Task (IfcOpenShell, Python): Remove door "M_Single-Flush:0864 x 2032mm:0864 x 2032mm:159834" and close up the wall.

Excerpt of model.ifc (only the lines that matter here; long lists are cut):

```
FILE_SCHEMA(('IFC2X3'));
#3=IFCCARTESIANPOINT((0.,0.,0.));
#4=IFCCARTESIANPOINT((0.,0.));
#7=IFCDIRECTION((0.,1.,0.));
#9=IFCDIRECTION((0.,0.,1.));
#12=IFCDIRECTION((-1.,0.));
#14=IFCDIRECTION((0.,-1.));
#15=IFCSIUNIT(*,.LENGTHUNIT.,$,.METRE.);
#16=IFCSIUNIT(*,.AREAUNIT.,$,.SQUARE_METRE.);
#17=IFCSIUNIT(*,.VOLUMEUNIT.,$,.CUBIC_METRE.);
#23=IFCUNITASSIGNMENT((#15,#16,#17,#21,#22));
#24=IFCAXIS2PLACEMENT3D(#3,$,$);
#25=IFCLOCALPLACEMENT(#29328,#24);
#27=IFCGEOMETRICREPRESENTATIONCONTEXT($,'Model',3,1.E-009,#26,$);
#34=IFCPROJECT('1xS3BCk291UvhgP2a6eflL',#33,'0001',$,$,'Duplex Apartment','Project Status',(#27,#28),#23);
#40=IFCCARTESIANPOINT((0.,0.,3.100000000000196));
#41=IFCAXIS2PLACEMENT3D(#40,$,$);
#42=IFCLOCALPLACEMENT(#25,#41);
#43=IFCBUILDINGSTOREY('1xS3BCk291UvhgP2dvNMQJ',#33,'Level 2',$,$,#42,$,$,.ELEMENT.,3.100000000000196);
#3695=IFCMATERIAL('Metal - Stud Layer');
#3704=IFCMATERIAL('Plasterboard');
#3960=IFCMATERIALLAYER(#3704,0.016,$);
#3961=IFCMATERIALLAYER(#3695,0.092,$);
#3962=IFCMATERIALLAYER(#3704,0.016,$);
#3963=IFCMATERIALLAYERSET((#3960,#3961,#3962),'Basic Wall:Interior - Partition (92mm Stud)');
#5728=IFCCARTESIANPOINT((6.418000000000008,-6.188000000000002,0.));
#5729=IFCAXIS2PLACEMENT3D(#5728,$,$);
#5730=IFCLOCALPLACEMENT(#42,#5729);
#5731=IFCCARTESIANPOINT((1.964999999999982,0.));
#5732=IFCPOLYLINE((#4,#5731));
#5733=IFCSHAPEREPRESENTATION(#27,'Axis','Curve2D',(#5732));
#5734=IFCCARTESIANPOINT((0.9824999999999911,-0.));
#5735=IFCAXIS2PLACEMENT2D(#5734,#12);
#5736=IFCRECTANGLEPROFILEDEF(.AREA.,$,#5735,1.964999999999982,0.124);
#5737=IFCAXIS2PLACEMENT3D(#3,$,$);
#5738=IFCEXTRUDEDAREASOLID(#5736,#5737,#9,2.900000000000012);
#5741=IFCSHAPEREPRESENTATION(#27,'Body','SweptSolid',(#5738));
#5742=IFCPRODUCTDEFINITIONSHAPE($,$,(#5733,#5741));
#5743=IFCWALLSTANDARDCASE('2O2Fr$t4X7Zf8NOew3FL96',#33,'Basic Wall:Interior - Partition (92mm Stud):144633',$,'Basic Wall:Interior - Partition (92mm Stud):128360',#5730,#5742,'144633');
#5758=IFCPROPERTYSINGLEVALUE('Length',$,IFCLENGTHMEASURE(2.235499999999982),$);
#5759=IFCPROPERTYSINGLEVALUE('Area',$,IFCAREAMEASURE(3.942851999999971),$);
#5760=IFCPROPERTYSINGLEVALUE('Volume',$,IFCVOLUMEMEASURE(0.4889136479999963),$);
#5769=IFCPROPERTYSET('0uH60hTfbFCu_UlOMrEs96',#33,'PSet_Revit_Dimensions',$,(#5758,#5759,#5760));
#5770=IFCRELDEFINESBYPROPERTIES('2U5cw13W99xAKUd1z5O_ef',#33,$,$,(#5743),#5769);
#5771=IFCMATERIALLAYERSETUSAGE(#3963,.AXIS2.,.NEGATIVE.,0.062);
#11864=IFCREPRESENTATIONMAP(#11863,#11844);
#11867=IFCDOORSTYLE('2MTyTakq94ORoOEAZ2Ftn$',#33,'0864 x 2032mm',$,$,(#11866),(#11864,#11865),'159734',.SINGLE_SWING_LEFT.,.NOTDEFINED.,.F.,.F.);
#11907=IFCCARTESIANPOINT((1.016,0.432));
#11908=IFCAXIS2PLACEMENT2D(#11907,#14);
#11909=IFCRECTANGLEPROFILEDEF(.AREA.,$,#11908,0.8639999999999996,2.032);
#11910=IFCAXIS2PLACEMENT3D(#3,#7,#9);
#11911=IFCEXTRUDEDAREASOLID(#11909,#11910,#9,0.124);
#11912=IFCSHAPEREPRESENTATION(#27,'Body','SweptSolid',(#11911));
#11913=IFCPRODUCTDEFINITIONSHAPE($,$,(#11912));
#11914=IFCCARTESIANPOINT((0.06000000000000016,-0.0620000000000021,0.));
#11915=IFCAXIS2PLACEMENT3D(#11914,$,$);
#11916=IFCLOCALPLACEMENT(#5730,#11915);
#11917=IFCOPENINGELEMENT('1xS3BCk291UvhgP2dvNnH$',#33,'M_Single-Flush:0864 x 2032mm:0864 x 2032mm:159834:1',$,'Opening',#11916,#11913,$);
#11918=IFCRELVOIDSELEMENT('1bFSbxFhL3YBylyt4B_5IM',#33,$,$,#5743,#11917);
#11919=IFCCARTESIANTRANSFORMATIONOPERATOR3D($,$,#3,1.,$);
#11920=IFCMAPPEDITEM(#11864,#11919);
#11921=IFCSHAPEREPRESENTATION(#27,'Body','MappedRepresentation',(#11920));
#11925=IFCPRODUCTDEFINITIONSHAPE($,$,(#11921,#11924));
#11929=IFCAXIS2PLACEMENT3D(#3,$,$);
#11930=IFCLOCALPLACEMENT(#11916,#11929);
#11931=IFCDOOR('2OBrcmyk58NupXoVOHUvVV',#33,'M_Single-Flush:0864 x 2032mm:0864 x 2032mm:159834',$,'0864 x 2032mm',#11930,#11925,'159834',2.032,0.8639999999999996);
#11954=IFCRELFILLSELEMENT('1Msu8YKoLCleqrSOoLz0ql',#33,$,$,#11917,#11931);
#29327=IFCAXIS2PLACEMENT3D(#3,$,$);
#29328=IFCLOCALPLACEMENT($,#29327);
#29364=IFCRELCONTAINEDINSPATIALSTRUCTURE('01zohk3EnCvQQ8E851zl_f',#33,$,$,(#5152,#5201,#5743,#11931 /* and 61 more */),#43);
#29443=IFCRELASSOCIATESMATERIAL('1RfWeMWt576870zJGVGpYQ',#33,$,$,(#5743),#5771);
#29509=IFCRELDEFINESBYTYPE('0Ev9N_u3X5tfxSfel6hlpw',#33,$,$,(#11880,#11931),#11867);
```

```python
import ifcopenshell
import ifcopenshell.api.feature
import ifcopenshell.api.pset
import ifcopenshell.api.root
import ifcopenshell.geom
import ifcopenshell.util.element
import ifcopenshell.util.shape
import ifcopenshell.util.unit

model = ifcopenshell.open("model.ifc")
area_scale = ifcopenshell.util.unit.calculate_unit_scale(model, "AREAUNIT")
volume_scale = ifcopenshell.util.unit.calculate_unit_scale(model, "VOLUMEUNIT")
settings = ifcopenshell.geom.settings()


def volume(element):
    """Net volume in cubic metres, openings subtracted."""
    shape = ifcopenshell.geom.create_shape(settings, element)
    return ifcopenshell.util.shape.get_volume(shape.geometry)


door = model.by_id(11931)
opening = door.FillsVoids[0].RelatingOpeningElement
wall = opening.VoidsElements[0].RelatingBuildingElement
before = volume(wall)

ifcopenshell.api.root.remove_product(model, product=door)
ifcopenshell.api.feature.remove_feature(model, feature=opening)

after = volume(wall)
thickness = 0.124  # wall thickness in metres

# Update the wall's stored quantities.
pset = model.by_id(ifcopenshell.util.element.get_pset(wall, "PSet_Revit_Dimensions", should_inherit=False)["id"])
ifcopenshell.api.pset.edit_pset(model, pset=pset, properties={
    "Area": model.create_entity("IfcAreaMeasure", after / thickness / area_scale),
    "Volume": model.create_entity("IfcVolumeMeasure", after / volume_scale),
})

print(f"wall volume {before:.3f} -> {after:.3f} m3")

model.write("model_edited.ifc")
```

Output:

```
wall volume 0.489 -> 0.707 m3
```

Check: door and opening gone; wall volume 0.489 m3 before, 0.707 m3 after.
